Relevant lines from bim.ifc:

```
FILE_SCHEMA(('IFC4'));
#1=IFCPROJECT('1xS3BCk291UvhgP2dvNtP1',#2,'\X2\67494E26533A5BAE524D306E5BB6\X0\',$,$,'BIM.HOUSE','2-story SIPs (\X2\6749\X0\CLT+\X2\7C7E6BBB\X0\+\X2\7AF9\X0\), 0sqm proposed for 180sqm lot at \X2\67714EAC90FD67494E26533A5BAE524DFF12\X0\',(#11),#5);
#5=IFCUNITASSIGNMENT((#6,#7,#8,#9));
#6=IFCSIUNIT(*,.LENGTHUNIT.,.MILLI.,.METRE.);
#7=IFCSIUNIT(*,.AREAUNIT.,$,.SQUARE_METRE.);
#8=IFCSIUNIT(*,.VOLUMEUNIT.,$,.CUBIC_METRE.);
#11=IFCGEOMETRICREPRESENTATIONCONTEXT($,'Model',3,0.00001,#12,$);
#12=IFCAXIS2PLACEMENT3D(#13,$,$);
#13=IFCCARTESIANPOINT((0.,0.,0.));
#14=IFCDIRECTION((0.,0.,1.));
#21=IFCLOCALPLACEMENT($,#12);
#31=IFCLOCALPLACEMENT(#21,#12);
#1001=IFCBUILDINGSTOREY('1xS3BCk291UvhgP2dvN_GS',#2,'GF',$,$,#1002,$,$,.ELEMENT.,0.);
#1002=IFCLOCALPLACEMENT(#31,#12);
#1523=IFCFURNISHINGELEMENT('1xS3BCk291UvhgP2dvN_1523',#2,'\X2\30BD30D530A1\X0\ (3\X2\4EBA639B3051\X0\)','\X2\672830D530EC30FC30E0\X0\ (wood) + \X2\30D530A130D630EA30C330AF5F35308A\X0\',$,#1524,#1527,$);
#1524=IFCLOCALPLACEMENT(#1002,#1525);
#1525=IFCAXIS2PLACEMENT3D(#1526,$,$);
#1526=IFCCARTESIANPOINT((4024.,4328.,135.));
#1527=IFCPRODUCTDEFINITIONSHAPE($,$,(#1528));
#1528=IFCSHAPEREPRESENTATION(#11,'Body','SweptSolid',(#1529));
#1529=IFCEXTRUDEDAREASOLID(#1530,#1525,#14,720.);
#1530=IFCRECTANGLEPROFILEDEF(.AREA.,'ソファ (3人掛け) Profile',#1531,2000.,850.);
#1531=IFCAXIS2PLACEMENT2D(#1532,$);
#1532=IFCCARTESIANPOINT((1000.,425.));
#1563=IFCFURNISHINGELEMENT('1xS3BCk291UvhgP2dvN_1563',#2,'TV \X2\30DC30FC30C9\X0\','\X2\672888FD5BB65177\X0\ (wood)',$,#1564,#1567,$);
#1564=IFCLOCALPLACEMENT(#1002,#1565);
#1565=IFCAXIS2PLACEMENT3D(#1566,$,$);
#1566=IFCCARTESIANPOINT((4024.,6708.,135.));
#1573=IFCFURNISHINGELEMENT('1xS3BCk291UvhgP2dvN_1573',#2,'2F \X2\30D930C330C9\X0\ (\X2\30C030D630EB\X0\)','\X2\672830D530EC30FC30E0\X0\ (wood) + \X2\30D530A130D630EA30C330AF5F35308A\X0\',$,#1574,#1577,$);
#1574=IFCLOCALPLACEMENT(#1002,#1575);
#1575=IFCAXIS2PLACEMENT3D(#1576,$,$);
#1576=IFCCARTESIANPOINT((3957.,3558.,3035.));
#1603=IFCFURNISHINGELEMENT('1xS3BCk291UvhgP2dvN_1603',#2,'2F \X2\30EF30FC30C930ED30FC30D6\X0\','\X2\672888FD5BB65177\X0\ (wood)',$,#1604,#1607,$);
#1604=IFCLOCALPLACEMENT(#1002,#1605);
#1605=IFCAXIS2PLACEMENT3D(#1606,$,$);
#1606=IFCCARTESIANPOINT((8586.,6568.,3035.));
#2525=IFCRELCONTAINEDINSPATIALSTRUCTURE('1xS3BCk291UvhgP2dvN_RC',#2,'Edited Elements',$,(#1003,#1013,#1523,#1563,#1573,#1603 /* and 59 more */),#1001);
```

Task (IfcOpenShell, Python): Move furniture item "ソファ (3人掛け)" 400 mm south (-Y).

```python
import ifcopenshell
import ifcopenshell.api.geometry
import ifcopenshell.util.placement
import ifcopenshell.util.unit

model = ifcopenshell.open("bim.ifc")
unit_scale = ifcopenshell.util.unit.calculate_unit_scale(model)

item = model.by_guid("1xS3BCk291UvhgP2dvN_1523")
matrix = ifcopenshell.util.placement.get_local_placement(item.ObjectPlacement)
matrix[1, 3] -= 0.4 / unit_scale
ifcopenshell.api.geometry.edit_object_placement(model, product=item, matrix=matrix, is_si=False)

print(ifcopenshell.util.placement.get_local_placement(item.ObjectPlacement).round(3) + 0.0)

model.write("bim_rev.ifc")
```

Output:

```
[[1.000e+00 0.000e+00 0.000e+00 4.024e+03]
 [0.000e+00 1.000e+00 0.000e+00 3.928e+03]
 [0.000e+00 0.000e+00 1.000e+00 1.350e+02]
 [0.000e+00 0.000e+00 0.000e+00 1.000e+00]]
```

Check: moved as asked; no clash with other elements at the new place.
